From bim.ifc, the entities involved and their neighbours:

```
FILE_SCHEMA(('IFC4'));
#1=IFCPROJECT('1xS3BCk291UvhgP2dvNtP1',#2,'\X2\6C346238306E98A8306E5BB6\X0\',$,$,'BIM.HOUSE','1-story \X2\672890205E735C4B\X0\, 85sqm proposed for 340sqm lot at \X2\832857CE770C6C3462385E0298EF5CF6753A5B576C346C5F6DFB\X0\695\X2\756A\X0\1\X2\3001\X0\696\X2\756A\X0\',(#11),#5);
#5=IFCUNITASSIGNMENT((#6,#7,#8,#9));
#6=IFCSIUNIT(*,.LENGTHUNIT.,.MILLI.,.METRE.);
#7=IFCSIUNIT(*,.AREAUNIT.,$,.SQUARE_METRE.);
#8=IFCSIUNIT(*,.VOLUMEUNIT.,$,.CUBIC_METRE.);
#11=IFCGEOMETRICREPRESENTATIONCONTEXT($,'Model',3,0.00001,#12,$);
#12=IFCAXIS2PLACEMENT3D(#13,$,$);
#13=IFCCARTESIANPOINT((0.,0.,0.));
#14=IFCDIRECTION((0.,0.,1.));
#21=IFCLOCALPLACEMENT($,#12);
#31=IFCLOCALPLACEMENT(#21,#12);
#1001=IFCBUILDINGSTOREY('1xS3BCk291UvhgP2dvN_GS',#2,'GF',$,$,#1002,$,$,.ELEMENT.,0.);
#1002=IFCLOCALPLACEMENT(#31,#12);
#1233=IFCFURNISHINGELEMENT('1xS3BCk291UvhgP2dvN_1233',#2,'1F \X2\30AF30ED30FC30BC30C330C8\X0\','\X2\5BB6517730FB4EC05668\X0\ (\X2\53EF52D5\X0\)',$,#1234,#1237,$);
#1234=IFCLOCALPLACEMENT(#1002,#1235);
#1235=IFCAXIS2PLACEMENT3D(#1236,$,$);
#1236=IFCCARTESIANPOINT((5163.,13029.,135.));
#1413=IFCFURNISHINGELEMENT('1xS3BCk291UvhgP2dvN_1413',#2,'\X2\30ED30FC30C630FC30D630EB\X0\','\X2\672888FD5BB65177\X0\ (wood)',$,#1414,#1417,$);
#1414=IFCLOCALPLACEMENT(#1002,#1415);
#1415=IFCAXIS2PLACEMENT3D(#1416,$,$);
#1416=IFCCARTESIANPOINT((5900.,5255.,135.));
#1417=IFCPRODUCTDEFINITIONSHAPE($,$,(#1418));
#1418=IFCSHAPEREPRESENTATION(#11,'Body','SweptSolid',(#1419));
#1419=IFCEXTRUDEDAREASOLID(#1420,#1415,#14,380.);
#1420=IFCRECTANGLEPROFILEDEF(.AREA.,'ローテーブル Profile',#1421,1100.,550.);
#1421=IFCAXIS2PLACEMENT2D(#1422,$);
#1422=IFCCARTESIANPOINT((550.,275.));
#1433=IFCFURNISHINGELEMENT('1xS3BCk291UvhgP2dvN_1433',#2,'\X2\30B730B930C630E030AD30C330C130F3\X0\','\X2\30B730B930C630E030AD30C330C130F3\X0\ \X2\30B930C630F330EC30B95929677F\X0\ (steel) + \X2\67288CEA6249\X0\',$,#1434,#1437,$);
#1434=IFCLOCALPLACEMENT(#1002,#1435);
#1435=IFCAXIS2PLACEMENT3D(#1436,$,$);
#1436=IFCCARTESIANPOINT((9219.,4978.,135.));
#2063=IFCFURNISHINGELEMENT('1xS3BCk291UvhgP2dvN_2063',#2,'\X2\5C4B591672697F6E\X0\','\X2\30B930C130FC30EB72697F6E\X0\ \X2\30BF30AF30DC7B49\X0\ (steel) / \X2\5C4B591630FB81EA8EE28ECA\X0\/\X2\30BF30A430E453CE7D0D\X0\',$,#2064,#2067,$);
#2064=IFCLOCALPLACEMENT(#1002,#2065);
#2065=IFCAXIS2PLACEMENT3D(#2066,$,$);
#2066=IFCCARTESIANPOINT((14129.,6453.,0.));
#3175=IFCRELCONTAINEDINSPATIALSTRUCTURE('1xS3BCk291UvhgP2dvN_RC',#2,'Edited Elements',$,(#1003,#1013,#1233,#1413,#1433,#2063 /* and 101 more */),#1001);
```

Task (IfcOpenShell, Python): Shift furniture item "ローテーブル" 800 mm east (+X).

```python
import ifcopenshell
import ifcopenshell.api.geometry
import ifcopenshell.util.placement

model = ifcopenshell.open("bim.ifc")

item = model.by_guid("1xS3BCk291UvhgP2dvN_1413")
matrix = ifcopenshell.util.placement.get_local_placement(item.ObjectPlacement)
matrix[0, 3] += 800.0
ifcopenshell.api.geometry.edit_object_placement(model, product=item, matrix=matrix, is_si=False)

print(ifcopenshell.util.placement.get_local_placement(item.ObjectPlacement).round(3) + 0.0)

model.write("bim_edited.ifc")
```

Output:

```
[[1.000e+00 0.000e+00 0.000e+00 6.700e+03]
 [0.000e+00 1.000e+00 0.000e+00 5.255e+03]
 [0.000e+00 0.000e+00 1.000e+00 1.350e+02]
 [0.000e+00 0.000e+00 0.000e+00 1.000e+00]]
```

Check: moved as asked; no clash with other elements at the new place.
